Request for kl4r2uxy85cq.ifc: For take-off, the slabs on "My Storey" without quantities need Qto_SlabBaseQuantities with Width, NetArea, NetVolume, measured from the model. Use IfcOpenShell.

First a look at what the model holds.

```python
import ifcopenshell
import ifcopenshell.util.element
import ifcopenshell.util.unit

model = ifcopenshell.open("kl4r2uxy85cq.ifc")
print(model.schema)
for unit_type in ("LENGTHUNIT", "AREAUNIT", "VOLUMEUNIT"):
    print(unit_type, ifcopenshell.util.unit.calculate_unit_scale(model, unit_type))
storey = next(s for s in model.by_type("IfcBuildingStorey") if s.Name == "My Storey")
slabs = [e for e in ifcopenshell.util.element.get_decomposition(storey) if e.is_a("IfcSlab")]
for e in sorted(slabs, key=lambda e: e.id()):
    print(e.id(), e.is_a(), e.Name, list(ifcopenshell.util.element.get_psets(e, qtos_only=True)), sep=" | ")
```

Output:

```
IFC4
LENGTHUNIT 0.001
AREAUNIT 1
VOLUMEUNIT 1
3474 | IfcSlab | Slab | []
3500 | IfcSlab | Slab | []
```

```python
import ifcopenshell
import ifcopenshell.api.pset
import ifcopenshell.geom
import ifcopenshell.util.element
import ifcopenshell.util.shape
import ifcopenshell.util.unit

model = ifcopenshell.open("kl4r2uxy85cq.ifc")
unit_scale = ifcopenshell.util.unit.calculate_unit_scale(model)
area_scale = ifcopenshell.util.unit.calculate_unit_scale(model, "AREAUNIT")
volume_scale = ifcopenshell.util.unit.calculate_unit_scale(model, "VOLUMEUNIT")
settings = ifcopenshell.geom.settings()

storey = next(s for s in model.by_type("IfcBuildingStorey") if s.Name == "My Storey")
slabs = [e for e in ifcopenshell.util.element.get_decomposition(storey) if e.is_a("IfcSlab")]

for e in sorted(slabs, key=lambda e: e.id()):
    if ifcopenshell.util.element.get_psets(e, qtos_only=True, should_inherit=False):
        continue
    # Geometry comes back in metres, in the element's own axes.
    shape = ifcopenshell.geom.create_shape(settings, e)
    values = {
        "Width": ifcopenshell.util.shape.get_z(shape.geometry) / unit_scale,
        "NetArea": ifcopenshell.util.shape.get_footprint_area(shape.geometry) / area_scale,
        "NetVolume": ifcopenshell.util.shape.get_volume(shape.geometry) / volume_scale,
    }
    qto = ifcopenshell.api.pset.add_qto(model, product=e, name="Qto_SlabBaseQuantities")
    ifcopenshell.api.pset.edit_qto(model, qto=qto, properties=values)
    print(e.id(), {k: round(v, 3) for k, v in values.items()})

model.write("kl4r2uxy85cq_rev.ifc")
```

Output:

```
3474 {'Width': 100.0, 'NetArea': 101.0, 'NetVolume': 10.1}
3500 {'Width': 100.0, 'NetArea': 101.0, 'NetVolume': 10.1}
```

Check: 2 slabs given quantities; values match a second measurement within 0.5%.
